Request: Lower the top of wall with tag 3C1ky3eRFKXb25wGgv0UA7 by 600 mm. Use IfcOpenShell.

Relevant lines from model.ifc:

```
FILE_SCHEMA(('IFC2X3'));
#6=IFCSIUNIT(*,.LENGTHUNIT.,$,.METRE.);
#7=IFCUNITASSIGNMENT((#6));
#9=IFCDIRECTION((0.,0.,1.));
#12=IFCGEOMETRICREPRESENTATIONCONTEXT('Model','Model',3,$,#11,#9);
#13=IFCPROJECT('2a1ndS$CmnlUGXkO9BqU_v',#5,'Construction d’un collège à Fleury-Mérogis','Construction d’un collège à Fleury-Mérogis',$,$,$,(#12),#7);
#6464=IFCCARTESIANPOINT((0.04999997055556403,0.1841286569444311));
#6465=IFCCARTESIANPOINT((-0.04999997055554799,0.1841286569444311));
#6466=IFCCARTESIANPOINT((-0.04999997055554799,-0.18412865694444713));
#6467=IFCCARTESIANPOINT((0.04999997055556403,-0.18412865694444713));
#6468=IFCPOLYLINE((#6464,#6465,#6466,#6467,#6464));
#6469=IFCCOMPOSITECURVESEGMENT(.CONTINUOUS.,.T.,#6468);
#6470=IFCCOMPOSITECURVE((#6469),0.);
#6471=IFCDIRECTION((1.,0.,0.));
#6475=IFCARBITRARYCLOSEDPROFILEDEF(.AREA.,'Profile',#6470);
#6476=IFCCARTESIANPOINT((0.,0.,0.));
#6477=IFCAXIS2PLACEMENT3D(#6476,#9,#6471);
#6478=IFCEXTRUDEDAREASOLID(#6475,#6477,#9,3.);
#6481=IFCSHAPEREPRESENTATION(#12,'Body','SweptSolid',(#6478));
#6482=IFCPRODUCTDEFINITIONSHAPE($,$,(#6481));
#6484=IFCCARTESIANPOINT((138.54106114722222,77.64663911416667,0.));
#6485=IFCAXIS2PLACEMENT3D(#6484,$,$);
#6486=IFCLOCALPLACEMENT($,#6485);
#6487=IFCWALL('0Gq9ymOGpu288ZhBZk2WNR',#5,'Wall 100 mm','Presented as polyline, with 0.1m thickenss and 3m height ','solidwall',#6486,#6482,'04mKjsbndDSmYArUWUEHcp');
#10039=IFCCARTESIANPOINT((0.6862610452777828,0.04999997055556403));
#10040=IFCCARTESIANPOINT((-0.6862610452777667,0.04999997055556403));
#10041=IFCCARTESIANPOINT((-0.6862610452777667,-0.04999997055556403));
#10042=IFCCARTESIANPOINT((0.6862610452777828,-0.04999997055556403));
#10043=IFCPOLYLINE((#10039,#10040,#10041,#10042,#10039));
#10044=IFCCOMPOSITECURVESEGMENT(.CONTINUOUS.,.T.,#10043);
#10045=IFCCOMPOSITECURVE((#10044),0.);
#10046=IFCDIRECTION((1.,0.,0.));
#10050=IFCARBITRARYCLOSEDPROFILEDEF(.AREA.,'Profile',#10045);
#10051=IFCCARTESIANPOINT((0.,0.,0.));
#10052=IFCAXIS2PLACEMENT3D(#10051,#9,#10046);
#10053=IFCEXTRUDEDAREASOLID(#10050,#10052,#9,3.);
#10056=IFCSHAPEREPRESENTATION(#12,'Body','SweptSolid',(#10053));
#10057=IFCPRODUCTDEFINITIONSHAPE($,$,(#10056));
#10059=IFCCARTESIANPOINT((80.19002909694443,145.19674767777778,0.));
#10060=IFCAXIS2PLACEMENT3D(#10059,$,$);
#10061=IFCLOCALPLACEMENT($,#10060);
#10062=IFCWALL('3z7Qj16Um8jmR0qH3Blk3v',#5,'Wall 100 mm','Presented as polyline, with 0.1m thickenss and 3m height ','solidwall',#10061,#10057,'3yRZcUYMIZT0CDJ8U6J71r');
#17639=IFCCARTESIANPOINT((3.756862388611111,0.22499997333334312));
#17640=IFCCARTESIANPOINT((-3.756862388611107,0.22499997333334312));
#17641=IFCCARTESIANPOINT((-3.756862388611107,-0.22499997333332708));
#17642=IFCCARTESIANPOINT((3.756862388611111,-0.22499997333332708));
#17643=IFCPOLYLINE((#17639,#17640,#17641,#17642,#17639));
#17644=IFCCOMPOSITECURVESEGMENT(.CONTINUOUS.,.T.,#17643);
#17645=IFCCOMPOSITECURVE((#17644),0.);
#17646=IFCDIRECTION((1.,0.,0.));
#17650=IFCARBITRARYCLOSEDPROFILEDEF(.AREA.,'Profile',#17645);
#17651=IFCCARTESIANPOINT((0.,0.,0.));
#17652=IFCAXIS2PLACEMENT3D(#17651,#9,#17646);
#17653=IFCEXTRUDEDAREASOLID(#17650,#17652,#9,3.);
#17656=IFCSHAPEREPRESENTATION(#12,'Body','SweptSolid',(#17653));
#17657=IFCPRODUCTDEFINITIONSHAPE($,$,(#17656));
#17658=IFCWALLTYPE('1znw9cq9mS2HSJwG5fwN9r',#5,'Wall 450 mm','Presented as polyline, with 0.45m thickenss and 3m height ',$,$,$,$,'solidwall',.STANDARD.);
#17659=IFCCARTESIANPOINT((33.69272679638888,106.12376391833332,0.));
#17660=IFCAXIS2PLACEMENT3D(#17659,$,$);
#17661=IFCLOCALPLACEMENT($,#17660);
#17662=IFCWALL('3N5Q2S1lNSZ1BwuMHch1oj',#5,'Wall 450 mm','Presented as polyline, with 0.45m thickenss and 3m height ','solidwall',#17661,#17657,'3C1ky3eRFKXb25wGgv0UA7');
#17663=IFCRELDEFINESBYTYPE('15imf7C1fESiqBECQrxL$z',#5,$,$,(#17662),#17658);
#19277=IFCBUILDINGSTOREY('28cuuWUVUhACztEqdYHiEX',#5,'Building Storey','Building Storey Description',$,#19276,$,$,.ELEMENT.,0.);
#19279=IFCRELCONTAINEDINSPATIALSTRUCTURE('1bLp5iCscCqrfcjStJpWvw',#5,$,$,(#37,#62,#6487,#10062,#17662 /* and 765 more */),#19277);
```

```python
import ifcopenshell
import ifcopenshell.geom
import ifcopenshell.util.shape

model = ifcopenshell.open("model.ifc")
settings = ifcopenshell.geom.settings()


def volume(element):
    """Net volume in cubic metres, openings subtracted."""
    shape = ifcopenshell.geom.create_shape(settings, element)
    return ifcopenshell.util.shape.get_volume(shape.geometry)


wall = model.by_guid("3N5Q2S1lNSZ1BwuMHch1oj")
before = volume(wall)

body = next(r for r in wall.Representation.Representations if r.RepresentationIdentifier == "Body")
solid = body.Items[0]
old_height = solid.Depth
solid.Depth -= 0.6
after = volume(wall)

print(f"height {old_height:g} -> {solid.Depth:g}, volume {before:.3f} -> {after:.3f} m3")

model.write("model_updated.ifc")
```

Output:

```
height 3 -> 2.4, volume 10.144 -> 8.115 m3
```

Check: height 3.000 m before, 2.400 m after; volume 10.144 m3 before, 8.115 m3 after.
